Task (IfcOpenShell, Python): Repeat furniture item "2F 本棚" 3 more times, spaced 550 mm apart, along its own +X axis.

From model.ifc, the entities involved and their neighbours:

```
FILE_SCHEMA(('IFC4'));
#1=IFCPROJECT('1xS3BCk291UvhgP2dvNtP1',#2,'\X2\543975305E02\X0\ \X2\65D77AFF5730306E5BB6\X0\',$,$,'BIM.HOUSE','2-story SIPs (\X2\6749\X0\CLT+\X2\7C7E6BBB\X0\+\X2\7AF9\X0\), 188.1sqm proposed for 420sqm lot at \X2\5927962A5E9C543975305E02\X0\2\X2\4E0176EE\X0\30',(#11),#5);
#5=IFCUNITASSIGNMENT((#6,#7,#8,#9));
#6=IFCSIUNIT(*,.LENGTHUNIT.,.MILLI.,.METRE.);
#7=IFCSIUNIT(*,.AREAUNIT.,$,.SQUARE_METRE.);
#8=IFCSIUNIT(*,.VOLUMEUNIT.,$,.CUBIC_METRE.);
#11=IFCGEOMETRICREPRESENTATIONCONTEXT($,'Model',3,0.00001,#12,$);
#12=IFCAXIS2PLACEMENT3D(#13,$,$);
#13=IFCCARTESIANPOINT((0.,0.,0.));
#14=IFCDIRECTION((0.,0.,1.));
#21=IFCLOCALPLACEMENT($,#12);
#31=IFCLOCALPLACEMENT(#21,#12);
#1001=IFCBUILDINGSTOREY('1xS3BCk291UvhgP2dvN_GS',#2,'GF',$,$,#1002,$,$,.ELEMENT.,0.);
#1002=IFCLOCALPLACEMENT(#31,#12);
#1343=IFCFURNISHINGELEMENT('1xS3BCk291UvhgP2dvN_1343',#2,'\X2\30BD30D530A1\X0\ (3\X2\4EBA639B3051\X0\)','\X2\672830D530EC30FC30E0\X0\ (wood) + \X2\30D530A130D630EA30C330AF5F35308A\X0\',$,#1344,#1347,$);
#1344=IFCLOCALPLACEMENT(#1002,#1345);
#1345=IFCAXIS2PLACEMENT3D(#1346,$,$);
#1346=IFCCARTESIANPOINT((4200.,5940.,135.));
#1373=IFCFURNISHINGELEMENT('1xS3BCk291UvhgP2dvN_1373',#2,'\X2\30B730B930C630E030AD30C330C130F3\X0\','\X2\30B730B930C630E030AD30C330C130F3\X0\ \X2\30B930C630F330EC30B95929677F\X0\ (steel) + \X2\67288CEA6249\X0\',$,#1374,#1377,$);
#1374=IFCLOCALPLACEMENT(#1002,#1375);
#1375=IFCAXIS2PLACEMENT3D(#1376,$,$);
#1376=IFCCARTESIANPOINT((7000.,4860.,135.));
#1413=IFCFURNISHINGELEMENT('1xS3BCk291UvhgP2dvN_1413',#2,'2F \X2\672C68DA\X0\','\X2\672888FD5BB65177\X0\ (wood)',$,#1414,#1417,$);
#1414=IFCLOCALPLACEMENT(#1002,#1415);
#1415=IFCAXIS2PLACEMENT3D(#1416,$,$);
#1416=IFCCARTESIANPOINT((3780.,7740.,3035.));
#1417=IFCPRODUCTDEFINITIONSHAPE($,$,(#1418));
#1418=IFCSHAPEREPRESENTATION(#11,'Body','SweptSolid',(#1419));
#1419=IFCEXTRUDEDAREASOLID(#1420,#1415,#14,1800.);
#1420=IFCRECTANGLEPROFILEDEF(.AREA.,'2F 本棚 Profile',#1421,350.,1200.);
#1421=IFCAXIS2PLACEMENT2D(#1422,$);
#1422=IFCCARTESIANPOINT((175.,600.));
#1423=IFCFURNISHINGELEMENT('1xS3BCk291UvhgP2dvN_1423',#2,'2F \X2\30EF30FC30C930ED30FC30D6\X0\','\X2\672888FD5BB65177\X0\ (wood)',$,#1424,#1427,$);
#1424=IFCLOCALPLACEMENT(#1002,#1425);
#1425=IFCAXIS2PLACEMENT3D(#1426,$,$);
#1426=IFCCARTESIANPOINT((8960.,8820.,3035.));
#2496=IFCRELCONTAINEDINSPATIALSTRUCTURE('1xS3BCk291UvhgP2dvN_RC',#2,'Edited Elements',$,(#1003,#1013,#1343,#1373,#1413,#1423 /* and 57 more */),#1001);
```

```python
import ifcopenshell
import ifcopenshell.api.geometry
import ifcopenshell.api.root
import ifcopenshell.util.element
import ifcopenshell.util.placement
import ifcopenshell.util.unit

model = ifcopenshell.open("model.ifc")
unit_scale = ifcopenshell.util.unit.calculate_unit_scale(model)


def reuse_history(source, copy):
    """copy_class also copies each property set's owner history, people and application; keep the originals."""
    for rel in copy.IsDefinedBy:
        if rel.is_a("IfcRelDefinesByProperties") and (history := rel.RelatingPropertyDefinition.OwnerHistory):
            rel.RelatingPropertyDefinition.OwnerHistory = source.OwnerHistory
            ifcopenshell.util.element.remove_deep2(model, history)


source = model.by_guid("1xS3BCk291UvhgP2dvN_1413")
base = ifcopenshell.util.placement.get_local_placement(source.ObjectPlacement)
step = base[:3, 0] * 0.55 / unit_scale

for i in range(1, 4):
    copy = ifcopenshell.api.root.copy_class(model, product=source)
    copy.Representation = ifcopenshell.util.element.copy_deep(
        model, source.Representation, exclude=["IfcGeometricRepresentationContext", "IfcRepresentationMap"]
    )
    reuse_history(source, copy)
    matrix = base.copy()
    matrix[:3, 3] += i * step
    print("added at", matrix[:3, 3].round(3) + 0.0)
    ifcopenshell.api.geometry.edit_object_placement(model, product=copy, matrix=matrix, is_si=False)

model.write("model_updated.ifc")
```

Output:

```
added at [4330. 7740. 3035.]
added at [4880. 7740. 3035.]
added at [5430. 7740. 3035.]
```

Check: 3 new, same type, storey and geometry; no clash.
